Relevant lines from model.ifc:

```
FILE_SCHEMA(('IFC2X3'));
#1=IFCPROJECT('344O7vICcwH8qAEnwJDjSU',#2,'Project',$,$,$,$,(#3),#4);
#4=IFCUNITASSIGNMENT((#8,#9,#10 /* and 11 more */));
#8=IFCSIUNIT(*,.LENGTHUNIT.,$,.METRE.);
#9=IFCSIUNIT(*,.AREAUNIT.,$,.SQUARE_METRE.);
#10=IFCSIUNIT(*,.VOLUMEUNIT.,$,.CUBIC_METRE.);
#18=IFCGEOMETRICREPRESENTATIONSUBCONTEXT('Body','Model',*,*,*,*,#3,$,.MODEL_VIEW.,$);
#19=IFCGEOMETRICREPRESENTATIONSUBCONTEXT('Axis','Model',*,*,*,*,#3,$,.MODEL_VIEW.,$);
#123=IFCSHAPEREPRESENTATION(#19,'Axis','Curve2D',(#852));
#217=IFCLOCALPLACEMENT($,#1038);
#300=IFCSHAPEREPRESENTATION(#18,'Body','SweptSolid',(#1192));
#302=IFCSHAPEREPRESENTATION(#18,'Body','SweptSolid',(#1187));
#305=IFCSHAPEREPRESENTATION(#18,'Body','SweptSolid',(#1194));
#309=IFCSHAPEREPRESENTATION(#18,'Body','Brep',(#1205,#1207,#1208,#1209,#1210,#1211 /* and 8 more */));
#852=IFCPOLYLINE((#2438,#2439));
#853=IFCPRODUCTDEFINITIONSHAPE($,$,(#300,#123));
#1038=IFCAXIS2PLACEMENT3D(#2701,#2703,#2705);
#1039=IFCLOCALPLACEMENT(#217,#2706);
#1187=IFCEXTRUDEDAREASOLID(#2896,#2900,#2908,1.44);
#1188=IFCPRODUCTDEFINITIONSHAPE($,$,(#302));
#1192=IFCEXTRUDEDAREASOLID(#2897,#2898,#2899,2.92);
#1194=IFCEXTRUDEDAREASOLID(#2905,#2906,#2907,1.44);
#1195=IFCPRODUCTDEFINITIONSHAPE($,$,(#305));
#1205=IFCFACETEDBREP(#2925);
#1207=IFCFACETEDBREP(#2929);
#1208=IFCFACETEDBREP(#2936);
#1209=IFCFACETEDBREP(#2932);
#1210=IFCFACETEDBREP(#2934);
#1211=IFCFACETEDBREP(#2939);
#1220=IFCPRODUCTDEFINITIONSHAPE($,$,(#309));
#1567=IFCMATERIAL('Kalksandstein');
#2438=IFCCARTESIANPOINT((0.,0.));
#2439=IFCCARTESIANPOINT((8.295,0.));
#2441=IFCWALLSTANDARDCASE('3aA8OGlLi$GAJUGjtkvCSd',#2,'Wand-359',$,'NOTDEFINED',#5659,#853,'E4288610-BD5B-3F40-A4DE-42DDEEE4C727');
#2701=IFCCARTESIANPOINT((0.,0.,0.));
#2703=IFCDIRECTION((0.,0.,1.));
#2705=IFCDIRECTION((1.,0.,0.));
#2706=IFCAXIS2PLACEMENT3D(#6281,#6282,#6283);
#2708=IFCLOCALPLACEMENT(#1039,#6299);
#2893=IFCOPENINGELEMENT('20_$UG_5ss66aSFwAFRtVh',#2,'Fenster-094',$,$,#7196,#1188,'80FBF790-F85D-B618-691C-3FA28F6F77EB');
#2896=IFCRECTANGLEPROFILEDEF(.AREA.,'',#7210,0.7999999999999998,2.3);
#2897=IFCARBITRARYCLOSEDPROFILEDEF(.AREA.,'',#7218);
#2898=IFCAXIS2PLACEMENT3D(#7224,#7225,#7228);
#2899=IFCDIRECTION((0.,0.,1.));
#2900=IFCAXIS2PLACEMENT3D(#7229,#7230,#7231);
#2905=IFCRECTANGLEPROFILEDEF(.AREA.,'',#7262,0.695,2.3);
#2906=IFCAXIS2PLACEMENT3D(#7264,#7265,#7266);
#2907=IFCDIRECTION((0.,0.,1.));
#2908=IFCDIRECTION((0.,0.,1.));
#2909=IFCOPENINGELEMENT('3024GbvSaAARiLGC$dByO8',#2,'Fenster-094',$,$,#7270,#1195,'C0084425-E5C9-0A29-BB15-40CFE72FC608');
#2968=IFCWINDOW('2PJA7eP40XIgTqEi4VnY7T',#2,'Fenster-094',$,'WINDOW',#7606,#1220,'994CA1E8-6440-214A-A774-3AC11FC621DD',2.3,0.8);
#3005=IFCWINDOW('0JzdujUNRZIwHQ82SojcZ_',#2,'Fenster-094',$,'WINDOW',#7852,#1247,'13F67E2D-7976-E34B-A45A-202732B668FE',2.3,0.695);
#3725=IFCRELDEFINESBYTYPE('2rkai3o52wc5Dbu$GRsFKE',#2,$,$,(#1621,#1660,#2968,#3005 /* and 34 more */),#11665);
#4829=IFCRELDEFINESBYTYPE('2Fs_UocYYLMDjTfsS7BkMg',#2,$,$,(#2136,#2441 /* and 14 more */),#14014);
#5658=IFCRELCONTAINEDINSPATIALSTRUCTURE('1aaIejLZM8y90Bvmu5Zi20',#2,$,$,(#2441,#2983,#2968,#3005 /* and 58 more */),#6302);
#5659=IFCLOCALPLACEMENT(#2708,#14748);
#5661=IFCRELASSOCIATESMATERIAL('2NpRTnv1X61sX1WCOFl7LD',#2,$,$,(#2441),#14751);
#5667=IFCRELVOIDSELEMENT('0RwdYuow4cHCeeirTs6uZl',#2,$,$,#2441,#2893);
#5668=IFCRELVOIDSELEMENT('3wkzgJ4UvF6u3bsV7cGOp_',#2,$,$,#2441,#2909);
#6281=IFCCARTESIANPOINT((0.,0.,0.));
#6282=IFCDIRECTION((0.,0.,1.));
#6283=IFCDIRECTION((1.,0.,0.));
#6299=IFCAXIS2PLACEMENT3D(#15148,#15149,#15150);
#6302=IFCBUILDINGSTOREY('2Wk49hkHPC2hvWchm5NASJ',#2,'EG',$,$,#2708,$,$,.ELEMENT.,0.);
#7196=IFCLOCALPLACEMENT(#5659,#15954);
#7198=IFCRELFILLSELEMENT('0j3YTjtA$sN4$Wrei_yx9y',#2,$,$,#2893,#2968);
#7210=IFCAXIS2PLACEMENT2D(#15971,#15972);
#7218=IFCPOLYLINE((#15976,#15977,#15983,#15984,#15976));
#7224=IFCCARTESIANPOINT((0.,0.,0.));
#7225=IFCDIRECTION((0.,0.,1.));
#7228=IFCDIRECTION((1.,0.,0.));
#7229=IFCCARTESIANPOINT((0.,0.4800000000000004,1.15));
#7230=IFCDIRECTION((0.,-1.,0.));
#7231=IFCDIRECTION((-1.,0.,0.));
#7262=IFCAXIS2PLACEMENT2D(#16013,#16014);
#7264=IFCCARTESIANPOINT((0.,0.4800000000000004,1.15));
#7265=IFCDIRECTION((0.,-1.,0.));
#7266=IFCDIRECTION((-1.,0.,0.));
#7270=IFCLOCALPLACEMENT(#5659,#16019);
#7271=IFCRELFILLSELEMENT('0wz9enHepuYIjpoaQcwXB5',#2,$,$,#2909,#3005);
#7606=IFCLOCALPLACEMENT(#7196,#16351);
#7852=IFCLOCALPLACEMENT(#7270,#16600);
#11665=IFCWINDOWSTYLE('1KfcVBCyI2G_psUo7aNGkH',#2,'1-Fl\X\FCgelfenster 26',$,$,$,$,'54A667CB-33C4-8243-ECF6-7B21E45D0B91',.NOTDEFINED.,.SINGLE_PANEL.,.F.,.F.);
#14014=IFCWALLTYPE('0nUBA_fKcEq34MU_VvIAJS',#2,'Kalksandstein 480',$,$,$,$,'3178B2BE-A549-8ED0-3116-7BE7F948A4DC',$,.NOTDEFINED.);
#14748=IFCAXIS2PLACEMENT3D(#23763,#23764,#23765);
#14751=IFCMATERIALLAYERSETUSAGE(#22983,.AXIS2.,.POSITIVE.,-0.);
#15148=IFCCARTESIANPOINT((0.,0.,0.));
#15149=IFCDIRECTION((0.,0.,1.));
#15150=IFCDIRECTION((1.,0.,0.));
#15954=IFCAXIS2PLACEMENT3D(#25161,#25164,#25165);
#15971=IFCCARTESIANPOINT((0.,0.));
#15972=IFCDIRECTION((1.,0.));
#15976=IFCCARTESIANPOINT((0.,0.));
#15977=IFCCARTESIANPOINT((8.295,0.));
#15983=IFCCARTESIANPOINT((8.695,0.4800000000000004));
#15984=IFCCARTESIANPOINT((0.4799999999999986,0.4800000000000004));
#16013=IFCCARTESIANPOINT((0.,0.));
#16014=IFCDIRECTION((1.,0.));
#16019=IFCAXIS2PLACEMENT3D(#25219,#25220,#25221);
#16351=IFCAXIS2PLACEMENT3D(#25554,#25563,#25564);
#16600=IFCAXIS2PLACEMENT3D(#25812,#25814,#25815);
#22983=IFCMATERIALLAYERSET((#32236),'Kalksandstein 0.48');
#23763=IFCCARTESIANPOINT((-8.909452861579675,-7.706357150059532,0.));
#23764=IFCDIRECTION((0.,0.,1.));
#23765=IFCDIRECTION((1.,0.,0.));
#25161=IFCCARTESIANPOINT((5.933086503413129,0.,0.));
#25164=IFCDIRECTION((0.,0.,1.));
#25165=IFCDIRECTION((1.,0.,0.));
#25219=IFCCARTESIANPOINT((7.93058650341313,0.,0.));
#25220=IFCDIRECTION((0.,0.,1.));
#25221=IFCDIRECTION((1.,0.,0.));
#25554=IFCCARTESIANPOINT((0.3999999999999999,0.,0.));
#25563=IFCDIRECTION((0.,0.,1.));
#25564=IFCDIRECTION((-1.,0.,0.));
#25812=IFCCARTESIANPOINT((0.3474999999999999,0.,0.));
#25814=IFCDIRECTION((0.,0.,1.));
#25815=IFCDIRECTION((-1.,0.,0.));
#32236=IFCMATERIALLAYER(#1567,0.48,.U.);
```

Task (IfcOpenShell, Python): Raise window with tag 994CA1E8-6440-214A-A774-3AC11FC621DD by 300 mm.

```python
import numpy as np
import ifcopenshell
import ifcopenshell.api.geometry
import ifcopenshell.util.placement
import ifcopenshell.util.unit

model = ifcopenshell.open("model.ifc")
unit_scale = ifcopenshell.util.unit.calculate_unit_scale(model)

window = model.by_guid("2PJA7eP40XIgTqEi4VnY7T")
opening = window.FillsVoids[0].RelatingOpeningElement
dz = 0.3

shift = np.array([0.0, 0.0, dz])
# The window is placed relative to its opening, so it follows when the opening moves.
matrix = ifcopenshell.util.placement.get_local_placement(opening.ObjectPlacement)
matrix[:3, 3] += shift
ifcopenshell.api.geometry.edit_object_placement(
    model, product=opening, matrix=matrix, is_si=False, should_transform_children=True
)

print(f"moved by {dz * unit_scale:+.3f} m")

model.write("model_v2.ifc")
```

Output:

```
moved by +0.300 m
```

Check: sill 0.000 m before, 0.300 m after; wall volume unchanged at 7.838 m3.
